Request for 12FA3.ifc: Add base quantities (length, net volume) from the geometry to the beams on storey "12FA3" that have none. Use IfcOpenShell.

First a look at what the model holds.

```python
import ifcopenshell
import ifcopenshell.util.element
import ifcopenshell.util.unit

model = ifcopenshell.open("12FA3.ifc")
print(model.schema)
for unit_type in ("LENGTHUNIT", "AREAUNIT", "VOLUMEUNIT"):
    print(unit_type, ifcopenshell.util.unit.calculate_unit_scale(model, unit_type))
storey = next(s for s in model.by_type("IfcBuildingStorey") if s.Name == "12FA3")
beams = [e for e in ifcopenshell.util.element.get_decomposition(storey) if e.is_a("IfcBeam")]
for e in sorted(beams, key=lambda e: e.id()):
    print(e.id(), e.is_a(), e.Name, list(ifcopenshell.util.element.get_psets(e, qtos_only=True)), sep=" | ")
```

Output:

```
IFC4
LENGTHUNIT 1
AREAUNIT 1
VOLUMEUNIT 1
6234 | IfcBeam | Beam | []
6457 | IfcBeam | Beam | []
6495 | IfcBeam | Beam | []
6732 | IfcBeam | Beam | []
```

```python
import ifcopenshell
import ifcopenshell.api.pset
import ifcopenshell.geom
import ifcopenshell.util.element
import ifcopenshell.util.shape
import ifcopenshell.util.unit

model = ifcopenshell.open("12FA3.ifc")
unit_scale = ifcopenshell.util.unit.calculate_unit_scale(model)
volume_scale = ifcopenshell.util.unit.calculate_unit_scale(model, "VOLUMEUNIT")
settings = ifcopenshell.geom.settings()

storey = next(s for s in model.by_type("IfcBuildingStorey") if s.Name == "12FA3")
beams = [e for e in ifcopenshell.util.element.get_decomposition(storey) if e.is_a("IfcBeam")]

for e in sorted(beams, key=lambda e: e.id()):
    if ifcopenshell.util.element.get_psets(e, qtos_only=True, should_inherit=False):
        continue
    # Geometry comes back in metres, in the element's own axes.
    shape = ifcopenshell.geom.create_shape(settings, e)
    values = {
        "Length": ifcopenshell.util.shape.get_max_xyz(shape.geometry) / unit_scale,
        "NetVolume": ifcopenshell.util.shape.get_volume(shape.geometry) / volume_scale,
    }
    qto = ifcopenshell.api.pset.add_qto(model, product=e, name="Qto_BeamBaseQuantities")
    ifcopenshell.api.pset.edit_qto(model, qto=qto, properties=values)
    print(e.id(), {k: round(v, 3) for k, v in values.items()})

model.write("12FA3_rev.ifc")
```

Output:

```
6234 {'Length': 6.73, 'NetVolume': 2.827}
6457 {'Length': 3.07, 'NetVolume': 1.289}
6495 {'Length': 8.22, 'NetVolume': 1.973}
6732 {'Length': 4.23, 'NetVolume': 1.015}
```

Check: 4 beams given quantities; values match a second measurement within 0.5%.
